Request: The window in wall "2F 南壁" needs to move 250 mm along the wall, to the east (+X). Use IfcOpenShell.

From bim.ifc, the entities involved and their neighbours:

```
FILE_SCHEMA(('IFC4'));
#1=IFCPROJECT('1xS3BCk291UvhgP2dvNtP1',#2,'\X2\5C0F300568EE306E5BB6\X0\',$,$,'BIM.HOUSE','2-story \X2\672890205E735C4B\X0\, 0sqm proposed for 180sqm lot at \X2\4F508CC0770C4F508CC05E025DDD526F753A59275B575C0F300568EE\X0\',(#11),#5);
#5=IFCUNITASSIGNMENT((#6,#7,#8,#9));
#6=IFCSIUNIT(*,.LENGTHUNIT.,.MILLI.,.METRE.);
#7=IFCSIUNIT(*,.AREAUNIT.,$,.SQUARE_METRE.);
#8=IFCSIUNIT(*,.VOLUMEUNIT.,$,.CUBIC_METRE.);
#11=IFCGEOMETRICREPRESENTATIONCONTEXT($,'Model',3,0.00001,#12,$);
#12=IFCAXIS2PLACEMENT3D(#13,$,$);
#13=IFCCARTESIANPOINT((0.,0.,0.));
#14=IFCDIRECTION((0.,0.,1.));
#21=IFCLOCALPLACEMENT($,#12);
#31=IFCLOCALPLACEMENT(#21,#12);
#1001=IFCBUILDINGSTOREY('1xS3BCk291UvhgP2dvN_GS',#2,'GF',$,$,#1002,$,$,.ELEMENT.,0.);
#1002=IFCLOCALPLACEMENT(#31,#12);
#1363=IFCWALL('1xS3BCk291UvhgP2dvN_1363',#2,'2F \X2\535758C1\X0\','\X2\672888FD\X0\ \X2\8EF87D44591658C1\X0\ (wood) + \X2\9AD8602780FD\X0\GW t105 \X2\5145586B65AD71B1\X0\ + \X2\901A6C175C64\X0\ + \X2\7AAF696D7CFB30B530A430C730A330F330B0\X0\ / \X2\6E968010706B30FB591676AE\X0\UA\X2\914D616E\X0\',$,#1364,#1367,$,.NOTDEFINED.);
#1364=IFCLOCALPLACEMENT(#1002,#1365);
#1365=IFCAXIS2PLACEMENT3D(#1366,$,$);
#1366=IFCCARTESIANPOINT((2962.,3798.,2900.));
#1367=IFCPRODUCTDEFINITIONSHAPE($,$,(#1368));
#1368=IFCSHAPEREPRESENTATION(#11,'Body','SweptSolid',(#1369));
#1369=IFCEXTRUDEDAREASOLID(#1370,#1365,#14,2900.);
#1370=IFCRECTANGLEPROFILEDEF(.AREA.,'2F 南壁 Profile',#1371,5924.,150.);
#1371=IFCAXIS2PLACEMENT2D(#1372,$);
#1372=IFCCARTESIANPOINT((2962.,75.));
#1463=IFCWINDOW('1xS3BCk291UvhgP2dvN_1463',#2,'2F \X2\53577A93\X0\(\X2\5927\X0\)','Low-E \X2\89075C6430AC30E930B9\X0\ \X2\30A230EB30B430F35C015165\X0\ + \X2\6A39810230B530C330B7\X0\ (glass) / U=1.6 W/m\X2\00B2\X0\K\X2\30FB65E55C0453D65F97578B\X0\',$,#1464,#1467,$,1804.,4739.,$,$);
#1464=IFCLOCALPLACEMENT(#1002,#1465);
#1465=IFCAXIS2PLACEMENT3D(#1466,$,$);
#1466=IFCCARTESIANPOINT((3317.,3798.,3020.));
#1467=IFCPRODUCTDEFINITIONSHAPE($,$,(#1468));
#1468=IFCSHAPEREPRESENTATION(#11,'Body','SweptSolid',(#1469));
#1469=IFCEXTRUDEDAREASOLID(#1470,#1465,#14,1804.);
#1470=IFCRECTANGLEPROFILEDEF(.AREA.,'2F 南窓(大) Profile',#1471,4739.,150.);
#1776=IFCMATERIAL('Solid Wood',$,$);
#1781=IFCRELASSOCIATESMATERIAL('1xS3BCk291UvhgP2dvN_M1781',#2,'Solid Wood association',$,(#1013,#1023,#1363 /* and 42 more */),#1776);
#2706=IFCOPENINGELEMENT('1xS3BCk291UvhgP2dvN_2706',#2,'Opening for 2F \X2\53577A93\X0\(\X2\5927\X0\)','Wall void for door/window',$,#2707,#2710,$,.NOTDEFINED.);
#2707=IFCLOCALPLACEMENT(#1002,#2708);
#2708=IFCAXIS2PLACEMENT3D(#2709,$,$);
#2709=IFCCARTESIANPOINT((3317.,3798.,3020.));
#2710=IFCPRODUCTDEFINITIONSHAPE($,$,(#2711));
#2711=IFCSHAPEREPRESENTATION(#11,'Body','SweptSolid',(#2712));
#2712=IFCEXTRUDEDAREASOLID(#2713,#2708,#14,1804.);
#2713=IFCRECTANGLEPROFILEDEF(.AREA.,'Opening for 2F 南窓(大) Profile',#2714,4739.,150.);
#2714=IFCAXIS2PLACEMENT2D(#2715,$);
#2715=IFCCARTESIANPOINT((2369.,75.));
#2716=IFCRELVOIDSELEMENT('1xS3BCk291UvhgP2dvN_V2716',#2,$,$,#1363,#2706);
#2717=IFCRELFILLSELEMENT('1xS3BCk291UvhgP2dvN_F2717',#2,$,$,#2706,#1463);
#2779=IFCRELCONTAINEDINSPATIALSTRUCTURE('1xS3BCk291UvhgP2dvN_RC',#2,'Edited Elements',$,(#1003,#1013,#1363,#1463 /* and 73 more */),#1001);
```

```python
import ifcopenshell
import ifcopenshell.api.geometry
import ifcopenshell.util.placement

model = ifcopenshell.open("bim.ifc")

window = model.by_guid("1xS3BCk291UvhgP2dvN_1463")
opening = window.FillsVoids[0].RelatingOpeningElement
wall = opening.VoidsElements[0].RelatingBuildingElement

wall_matrix = ifcopenshell.util.placement.get_local_placement(wall.ObjectPlacement)
shift = wall_matrix[:3, 0] * 250.0
before = ifcopenshell.util.placement.get_local_placement(window.ObjectPlacement)[:3, 3].copy()

# The window is not placed relative to its opening, so move both.
for product in (opening, window):
    matrix = ifcopenshell.util.placement.get_local_placement(product.ObjectPlacement)
    matrix[:3, 3] += shift
    ifcopenshell.api.geometry.edit_object_placement(model, product=product, matrix=matrix, is_si=False)

after = ifcopenshell.util.placement.get_local_placement(window.ObjectPlacement)[:3, 3]
print("window moved by", (after - before).round(3) + 0.0)

model.write("bim_rev.ifc")
```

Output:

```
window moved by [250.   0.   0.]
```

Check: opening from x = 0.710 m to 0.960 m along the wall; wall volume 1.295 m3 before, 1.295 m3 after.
